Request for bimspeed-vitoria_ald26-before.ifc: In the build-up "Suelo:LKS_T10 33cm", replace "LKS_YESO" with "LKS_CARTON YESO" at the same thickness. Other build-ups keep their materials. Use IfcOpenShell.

First a look at what the model holds.

```python
import ifcopenshell
import ifcopenshell.util.element

model = ifcopenshell.open("bimspeed-vitoria_ald26-before.ifc")
print(model.schema)
for layer_set in model.by_type("IfcMaterialLayerSet"):
    if layer_set.LayerSetName == "Suelo:LKS_T10 33cm":
        for layer in layer_set.MaterialLayers:
            print(layer.id(), layer.Material and layer.Material.Name, layer.LayerThickness, sep=" | ")
        print(len(ifcopenshell.util.element.get_elements_by_material(model, layer_set)), "elements and types use it")
print(sorted(m.Name for m in model.by_type("IfcMaterial") if m.Name)[:60])
```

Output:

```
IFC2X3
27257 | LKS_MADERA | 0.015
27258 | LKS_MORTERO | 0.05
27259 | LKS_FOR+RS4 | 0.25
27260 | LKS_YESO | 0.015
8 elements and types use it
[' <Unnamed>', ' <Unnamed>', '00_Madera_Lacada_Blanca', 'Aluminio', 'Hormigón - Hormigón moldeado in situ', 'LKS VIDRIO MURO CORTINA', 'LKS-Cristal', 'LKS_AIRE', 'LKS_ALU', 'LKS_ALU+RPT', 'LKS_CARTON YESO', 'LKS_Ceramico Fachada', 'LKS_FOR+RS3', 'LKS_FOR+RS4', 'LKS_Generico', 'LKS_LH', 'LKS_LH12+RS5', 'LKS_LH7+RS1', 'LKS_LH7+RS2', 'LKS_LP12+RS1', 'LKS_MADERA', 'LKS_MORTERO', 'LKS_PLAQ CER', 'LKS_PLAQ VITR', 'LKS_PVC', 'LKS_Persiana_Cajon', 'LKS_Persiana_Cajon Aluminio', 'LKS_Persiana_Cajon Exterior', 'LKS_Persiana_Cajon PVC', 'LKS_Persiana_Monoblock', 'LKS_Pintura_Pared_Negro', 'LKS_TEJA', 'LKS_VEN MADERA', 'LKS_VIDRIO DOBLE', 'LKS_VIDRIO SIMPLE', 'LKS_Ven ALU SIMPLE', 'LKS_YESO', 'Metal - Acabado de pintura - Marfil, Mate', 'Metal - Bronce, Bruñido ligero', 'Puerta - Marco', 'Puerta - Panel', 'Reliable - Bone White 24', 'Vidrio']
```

```python
import ifcopenshell
import ifcopenshell.api.material

model = ifcopenshell.open("bimspeed-vitoria_ald26-before.ifc")

layer_set = next(s for s in model.by_type("IfcMaterialLayerSet") if s.LayerSetName == "Suelo:LKS_T10 33cm")
layer = next(l for l in layer_set.MaterialLayers if l.Material and l.Material.Name == "LKS_YESO")
material = next(m for m in model.by_type("IfcMaterial") if m.Name == "LKS_CARTON YESO")

# Point this one layer at the other material; renaming the old one would change it everywhere.
ifcopenshell.api.material.edit_layer(model, layer=layer, attributes={}, material=material)

print([l.Material.Name if l.Material else None for l in layer_set.MaterialLayers])

model.write("bimspeed-vitoria_ald26-before_rev.ifc")
```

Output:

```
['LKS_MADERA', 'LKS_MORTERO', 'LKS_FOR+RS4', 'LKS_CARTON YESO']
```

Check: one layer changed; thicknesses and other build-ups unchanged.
